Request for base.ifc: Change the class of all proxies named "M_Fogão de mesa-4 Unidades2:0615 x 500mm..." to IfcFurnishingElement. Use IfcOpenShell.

First a look at what the model holds.

```python
import re

import ifcopenshell

model = ifcopenshell.open("base.ifc")
print(model.schema)
seen = {}
for e in model.by_type("IfcBuildingElementProxy"):
    name = re.sub(r":\d+(:\d+)?$", "", e.Name or "")  # drop the element id that some exporters append
    seen[name] = seen.get(name, 0) + 1
for name, count in sorted(seen.items()):
    print(count, "x", name)
```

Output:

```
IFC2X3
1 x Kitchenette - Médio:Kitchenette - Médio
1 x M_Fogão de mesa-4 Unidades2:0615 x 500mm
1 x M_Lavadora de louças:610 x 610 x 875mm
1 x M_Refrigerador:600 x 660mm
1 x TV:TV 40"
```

```python
import ifcopenshell
import ifcopenshell.api.root

model = ifcopenshell.open("base.ifc")

proxies = [e.id() for e in model.by_type("IfcBuildingElementProxy") if (e.Name or "").startswith("M_Fogão de mesa-4 Unidades2:0615 x 500mm")]
for step_id in proxies:
    proxy = model.by_id(step_id)
    # Reclassifying a typed element also reclassifies its type and the type's other occurrences.
    if proxy.is_a("IfcBuildingElementProxy"):
        ifcopenshell.api.root.reassign_class(model, product=proxy, ifc_class="IfcFurnishingElement")

print(sum(model.by_id(i).is_a("IfcFurnishingElement") for i in proxies), "reclassified")

model.write("base_v2.ifc")
```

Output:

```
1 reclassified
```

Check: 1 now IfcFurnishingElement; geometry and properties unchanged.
